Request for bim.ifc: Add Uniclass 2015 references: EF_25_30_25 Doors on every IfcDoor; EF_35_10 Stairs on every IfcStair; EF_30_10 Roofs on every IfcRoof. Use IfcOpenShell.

First a look at what the model holds.

```python
import ifcopenshell

model = ifcopenshell.open("bim.ifc")
print(model.schema)
print("classifications:", [c.Name for c in model.by_type("IfcClassification")])
for ifc_class in ("IfcDoor", "IfcRoof", "IfcStair", "IfcWall", "IfcWindow"):
    print(ifc_class, len(model.by_type(ifc_class)))
```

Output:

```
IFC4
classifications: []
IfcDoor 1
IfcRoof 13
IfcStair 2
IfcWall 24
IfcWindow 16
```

```python
import ifcopenshell
import ifcopenshell.api.classification

model = ifcopenshell.open("bim.ifc")

system = ifcopenshell.api.classification.add_classification(model, classification="Uniclass 2015")

codes = {
    "IfcDoor": ("EF_25_30_25", "Doors"),
    "IfcStair": ("EF_35_10", "Stairs"),
    "IfcRoof": ("EF_30_10", "Roofs"),
}
for ifc_class, (code, name) in codes.items():
    products = model.by_type(ifc_class)
    ifcopenshell.api.classification.add_reference(
        model, products=products, classification=system, identification=code, name=name
    )
    print(code, len(products))

model.write("bim_v2.ifc")
```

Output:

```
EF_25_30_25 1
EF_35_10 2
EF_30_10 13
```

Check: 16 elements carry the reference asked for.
